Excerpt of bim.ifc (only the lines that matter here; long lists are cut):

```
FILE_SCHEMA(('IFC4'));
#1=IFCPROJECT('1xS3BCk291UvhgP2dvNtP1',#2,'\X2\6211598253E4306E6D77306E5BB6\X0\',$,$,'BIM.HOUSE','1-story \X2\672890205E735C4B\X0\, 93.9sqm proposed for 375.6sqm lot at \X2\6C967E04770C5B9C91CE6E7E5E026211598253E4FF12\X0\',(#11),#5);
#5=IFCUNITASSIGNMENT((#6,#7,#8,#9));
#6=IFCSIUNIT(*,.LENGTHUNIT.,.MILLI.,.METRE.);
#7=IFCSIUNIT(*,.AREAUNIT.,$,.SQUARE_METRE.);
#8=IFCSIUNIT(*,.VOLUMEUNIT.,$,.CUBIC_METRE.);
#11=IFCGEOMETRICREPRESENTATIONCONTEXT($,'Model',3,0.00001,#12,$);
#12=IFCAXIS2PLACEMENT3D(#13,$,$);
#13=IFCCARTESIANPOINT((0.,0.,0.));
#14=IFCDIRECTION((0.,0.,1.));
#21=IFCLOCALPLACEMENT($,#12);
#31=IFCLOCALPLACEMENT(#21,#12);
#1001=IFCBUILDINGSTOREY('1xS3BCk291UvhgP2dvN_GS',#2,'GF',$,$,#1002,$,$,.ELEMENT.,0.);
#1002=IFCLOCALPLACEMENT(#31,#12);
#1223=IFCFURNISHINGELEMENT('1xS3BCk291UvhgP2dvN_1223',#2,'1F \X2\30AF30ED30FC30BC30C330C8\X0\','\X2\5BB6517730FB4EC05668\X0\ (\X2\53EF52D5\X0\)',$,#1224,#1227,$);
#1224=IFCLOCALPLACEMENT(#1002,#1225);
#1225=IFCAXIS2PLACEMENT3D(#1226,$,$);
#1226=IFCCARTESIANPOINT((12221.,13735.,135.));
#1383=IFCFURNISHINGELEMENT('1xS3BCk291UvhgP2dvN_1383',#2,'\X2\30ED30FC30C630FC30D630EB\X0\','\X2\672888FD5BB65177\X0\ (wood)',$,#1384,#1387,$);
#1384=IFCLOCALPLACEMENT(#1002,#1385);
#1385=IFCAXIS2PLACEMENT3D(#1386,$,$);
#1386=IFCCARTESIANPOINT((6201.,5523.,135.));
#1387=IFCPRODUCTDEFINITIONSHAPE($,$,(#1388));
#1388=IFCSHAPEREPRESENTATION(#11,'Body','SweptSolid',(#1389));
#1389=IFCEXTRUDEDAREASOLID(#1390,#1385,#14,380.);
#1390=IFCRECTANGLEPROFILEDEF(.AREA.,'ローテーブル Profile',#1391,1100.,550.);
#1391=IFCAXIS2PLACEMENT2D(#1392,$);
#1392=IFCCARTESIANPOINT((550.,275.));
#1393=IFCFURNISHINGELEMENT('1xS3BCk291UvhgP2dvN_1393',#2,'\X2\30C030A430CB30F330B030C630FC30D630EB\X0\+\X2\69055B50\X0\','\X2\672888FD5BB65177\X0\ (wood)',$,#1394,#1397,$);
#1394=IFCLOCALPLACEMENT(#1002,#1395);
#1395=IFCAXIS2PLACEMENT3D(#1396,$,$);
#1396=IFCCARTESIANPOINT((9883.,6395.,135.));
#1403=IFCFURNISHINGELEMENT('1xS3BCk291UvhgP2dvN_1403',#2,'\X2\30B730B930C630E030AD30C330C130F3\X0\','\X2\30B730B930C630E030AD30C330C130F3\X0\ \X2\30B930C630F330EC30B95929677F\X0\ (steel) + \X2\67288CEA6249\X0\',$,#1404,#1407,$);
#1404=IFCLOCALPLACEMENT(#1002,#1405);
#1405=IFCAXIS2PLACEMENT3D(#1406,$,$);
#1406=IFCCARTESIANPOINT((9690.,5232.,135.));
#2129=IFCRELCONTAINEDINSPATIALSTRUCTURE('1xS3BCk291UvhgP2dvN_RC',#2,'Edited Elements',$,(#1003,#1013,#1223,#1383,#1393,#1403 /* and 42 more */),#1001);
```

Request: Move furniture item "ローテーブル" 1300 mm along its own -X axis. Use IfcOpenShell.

```python
import ifcopenshell
import ifcopenshell.api.geometry
import ifcopenshell.util.placement

model = ifcopenshell.open("bim.ifc")

item = model.by_guid("1xS3BCk291UvhgP2dvN_1383")
matrix = ifcopenshell.util.placement.get_local_placement(item.ObjectPlacement)
matrix[:3, 3] -= matrix[:3, 0] * 1300.0
ifcopenshell.api.geometry.edit_object_placement(model, product=item, matrix=matrix, is_si=False)

print(ifcopenshell.util.placement.get_local_placement(item.ObjectPlacement).round(3) + 0.0)

model.write("bim_rev.ifc")
```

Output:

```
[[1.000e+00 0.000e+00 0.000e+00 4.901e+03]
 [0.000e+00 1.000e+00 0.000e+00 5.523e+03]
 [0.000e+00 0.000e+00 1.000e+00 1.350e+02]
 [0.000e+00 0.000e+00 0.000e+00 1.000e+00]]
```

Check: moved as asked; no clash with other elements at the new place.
